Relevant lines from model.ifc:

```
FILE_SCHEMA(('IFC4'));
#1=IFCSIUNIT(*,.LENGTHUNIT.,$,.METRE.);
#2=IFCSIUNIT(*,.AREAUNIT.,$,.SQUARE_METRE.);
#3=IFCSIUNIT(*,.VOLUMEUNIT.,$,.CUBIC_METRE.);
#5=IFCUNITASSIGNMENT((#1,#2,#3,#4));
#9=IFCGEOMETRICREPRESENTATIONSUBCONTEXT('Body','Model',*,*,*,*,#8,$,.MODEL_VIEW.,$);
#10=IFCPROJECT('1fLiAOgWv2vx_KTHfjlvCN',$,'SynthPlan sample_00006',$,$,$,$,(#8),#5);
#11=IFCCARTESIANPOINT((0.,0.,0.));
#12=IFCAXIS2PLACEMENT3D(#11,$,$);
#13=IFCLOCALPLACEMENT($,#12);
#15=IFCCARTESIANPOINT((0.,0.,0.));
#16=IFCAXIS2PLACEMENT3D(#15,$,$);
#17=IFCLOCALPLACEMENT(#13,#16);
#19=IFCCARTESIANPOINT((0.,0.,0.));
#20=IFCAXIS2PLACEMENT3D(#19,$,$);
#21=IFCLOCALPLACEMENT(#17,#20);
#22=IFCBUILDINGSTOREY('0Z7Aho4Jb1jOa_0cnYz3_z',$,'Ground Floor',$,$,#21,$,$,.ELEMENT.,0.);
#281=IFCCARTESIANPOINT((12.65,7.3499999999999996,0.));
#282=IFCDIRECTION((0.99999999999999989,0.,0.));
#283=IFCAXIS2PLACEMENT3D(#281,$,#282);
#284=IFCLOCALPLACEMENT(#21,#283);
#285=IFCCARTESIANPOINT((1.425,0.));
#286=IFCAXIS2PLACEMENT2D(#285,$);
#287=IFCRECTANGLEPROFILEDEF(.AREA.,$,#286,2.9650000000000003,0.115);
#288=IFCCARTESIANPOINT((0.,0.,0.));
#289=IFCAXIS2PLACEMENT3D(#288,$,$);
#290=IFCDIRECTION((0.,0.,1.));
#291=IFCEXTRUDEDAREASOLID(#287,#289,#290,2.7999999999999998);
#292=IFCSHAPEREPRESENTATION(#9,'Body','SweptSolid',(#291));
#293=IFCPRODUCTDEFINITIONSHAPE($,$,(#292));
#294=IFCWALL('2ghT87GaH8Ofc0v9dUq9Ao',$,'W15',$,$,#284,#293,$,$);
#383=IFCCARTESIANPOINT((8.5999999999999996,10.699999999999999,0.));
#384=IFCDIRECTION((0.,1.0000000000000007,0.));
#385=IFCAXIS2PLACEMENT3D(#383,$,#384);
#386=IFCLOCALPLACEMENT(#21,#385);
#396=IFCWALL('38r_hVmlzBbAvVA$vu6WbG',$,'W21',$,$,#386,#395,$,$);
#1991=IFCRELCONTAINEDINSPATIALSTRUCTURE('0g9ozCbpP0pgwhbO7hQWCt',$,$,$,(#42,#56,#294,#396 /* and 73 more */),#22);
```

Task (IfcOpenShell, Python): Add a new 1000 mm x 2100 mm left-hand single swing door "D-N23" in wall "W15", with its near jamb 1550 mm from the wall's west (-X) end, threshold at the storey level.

```python
import numpy as np
import ifcopenshell
import ifcopenshell.api.feature
import ifcopenshell.api.geometry
import ifcopenshell.api.root
import ifcopenshell.api.spatial
import ifcopenshell.geom
import ifcopenshell.util.element
import ifcopenshell.util.placement
import ifcopenshell.util.representation
import ifcopenshell.util.shape
import ifcopenshell.util.unit

model = ifcopenshell.open("model.ifc")
unit_scale = ifcopenshell.util.unit.calculate_unit_scale(model)
settings = ifcopenshell.geom.settings()


def volume(element):
    """Net volume in cubic metres, openings subtracted."""
    shape = ifcopenshell.geom.create_shape(settings, element)
    return ifcopenshell.util.shape.get_volume(shape.geometry)


wall = model.by_id(294)
storey = ifcopenshell.util.element.get_container(wall, ifc_class="IfcBuildingStorey")
context = ifcopenshell.util.representation.get_context(model, "Model", "Body", "MODEL_VIEW")
before = volume(wall)

width, height, from_end, sill = 1, 2.1, 1.55, 0.0  # metres

# The wall runs along its own X axis, and the end named is its -X end.
wall_shape = ifcopenshell.geom.create_shape(settings, wall)
x, y, z = ifcopenshell.util.shape.get_vertices(wall_shape.geometry).T
start = x.min() + from_end
face, thickness = float(y.min()), float(y.max() - y.min())
wall_matrix = ifcopenshell.util.placement.get_local_placement(wall.ObjectPlacement)
level = ifcopenshell.util.placement.get_local_placement(storey.ObjectPlacement)[2, 3]


def in_wall(x, y):
    """Placement at x, y metres in the wall's axes, at sill height."""
    matrix = wall_matrix.copy()
    matrix[:, 3] = wall_matrix @ np.array([x / unit_scale, y / unit_scale, 0.0, 1.0])
    matrix[2, 3] = level + sill / unit_scale
    return matrix


# Opening: a box that overshoots both wall faces by 50 mm.
opening = ifcopenshell.api.root.create_entity(model, ifc_class="IfcOpeningElement", predefined_type="OPENING")
box = ifcopenshell.api.geometry.add_wall_representation(
    model, context=context, length=width, height=height, thickness=thickness + 0.1
)
ifcopenshell.api.geometry.assign_representation(model, product=opening, representation=box)
ifcopenshell.api.geometry.edit_object_placement(model, product=opening, matrix=in_wall(start, face - 0.05), is_si=False)
ifcopenshell.api.feature.add_feature(model, feature=opening, element=wall)

door = ifcopenshell.api.root.create_entity(model, ifc_class="IfcDoor", name="D-N23", predefined_type="DOOR")
door.OverallWidth, door.OverallHeight = width / unit_scale, height / unit_scale
door.OperationType = "SINGLE_SWING_LEFT"
body = ifcopenshell.api.geometry.add_door_representation(
    model,
    context=context,
    overall_width=door.OverallWidth,
    overall_height=door.OverallHeight,
    operation_type="SINGLE_SWING_LEFT",
    lining_properties={"LiningDepth": thickness / unit_scale, "ThresholdDepth": thickness / unit_scale},
)
ifcopenshell.api.geometry.assign_representation(model, product=door, representation=body)
ifcopenshell.api.spatial.assign_container(model, products=[door], relating_structure=storey)
ifcopenshell.api.feature.add_filling(model, opening=opening, element=door)

# The lining spans the wall, so the door starts at the wall face.
ifcopenshell.api.geometry.edit_object_placement(model, product=door, matrix=in_wall(start, face), is_si=False)

after = volume(wall)

print(f"wall volume {before:.3f} -> {after:.3f} m3")

model.write("model_v2.ifc")
```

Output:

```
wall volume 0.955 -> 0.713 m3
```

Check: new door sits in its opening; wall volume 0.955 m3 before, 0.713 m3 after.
